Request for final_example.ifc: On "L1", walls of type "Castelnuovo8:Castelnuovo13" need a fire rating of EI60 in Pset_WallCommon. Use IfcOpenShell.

First a look at what the model holds.

```python
import ifcopenshell
import ifcopenshell.util.element

model = ifcopenshell.open("final_example.ifc")
print(model.schema)
storey = next(s for s in model.by_type("IfcBuildingStorey") if s.Name == "L1")
walls = [e for e in ifcopenshell.util.element.get_decomposition(storey) if e.is_a("IfcWall")]
seen = {}
for e in walls:
    element_type = ifcopenshell.util.element.get_type(e)
    key = (element_type.Name if element_type != e and element_type else None, ifcopenshell.util.element.get_pset(e, "Pset_WallCommon", "FireRating"))
    seen[key] = seen.get(key, 0) + 1
for (name, value), count in sorted(seen.items(), key=str):
    print(count, "x", name, "|", value)
```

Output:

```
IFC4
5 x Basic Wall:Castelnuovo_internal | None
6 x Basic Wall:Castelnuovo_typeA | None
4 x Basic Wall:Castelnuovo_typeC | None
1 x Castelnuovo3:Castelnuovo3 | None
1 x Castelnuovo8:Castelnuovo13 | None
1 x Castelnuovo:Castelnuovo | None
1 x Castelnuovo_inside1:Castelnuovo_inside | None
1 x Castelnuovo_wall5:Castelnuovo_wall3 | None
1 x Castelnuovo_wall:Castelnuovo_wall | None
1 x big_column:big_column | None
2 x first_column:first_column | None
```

```python
import ifcopenshell
import ifcopenshell.api.pset
import ifcopenshell.util.element

model = ifcopenshell.open("final_example.ifc")

storey = next(s for s in model.by_type("IfcBuildingStorey") if s.Name == "L1")
walls = [e for e in ifcopenshell.util.element.get_decomposition(storey) if e.is_a("IfcWall")]

count = 0
for e in walls:
    element_type = ifcopenshell.util.element.get_type(e)
    if element_type in (None, e) or element_type.Name != "Castelnuovo8:Castelnuovo13":
        continue
    # add_pset returns the element's existing set when there is one.
    pset = ifcopenshell.api.pset.add_pset(model, product=e, name="Pset_WallCommon")
    ifcopenshell.api.pset.edit_pset(model, pset=pset, properties={"FireRating": "EI60"})
    count += 1

print(count, "walls updated")

model.write("final_example_v2.ifc")
```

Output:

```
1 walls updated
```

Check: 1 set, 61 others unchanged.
